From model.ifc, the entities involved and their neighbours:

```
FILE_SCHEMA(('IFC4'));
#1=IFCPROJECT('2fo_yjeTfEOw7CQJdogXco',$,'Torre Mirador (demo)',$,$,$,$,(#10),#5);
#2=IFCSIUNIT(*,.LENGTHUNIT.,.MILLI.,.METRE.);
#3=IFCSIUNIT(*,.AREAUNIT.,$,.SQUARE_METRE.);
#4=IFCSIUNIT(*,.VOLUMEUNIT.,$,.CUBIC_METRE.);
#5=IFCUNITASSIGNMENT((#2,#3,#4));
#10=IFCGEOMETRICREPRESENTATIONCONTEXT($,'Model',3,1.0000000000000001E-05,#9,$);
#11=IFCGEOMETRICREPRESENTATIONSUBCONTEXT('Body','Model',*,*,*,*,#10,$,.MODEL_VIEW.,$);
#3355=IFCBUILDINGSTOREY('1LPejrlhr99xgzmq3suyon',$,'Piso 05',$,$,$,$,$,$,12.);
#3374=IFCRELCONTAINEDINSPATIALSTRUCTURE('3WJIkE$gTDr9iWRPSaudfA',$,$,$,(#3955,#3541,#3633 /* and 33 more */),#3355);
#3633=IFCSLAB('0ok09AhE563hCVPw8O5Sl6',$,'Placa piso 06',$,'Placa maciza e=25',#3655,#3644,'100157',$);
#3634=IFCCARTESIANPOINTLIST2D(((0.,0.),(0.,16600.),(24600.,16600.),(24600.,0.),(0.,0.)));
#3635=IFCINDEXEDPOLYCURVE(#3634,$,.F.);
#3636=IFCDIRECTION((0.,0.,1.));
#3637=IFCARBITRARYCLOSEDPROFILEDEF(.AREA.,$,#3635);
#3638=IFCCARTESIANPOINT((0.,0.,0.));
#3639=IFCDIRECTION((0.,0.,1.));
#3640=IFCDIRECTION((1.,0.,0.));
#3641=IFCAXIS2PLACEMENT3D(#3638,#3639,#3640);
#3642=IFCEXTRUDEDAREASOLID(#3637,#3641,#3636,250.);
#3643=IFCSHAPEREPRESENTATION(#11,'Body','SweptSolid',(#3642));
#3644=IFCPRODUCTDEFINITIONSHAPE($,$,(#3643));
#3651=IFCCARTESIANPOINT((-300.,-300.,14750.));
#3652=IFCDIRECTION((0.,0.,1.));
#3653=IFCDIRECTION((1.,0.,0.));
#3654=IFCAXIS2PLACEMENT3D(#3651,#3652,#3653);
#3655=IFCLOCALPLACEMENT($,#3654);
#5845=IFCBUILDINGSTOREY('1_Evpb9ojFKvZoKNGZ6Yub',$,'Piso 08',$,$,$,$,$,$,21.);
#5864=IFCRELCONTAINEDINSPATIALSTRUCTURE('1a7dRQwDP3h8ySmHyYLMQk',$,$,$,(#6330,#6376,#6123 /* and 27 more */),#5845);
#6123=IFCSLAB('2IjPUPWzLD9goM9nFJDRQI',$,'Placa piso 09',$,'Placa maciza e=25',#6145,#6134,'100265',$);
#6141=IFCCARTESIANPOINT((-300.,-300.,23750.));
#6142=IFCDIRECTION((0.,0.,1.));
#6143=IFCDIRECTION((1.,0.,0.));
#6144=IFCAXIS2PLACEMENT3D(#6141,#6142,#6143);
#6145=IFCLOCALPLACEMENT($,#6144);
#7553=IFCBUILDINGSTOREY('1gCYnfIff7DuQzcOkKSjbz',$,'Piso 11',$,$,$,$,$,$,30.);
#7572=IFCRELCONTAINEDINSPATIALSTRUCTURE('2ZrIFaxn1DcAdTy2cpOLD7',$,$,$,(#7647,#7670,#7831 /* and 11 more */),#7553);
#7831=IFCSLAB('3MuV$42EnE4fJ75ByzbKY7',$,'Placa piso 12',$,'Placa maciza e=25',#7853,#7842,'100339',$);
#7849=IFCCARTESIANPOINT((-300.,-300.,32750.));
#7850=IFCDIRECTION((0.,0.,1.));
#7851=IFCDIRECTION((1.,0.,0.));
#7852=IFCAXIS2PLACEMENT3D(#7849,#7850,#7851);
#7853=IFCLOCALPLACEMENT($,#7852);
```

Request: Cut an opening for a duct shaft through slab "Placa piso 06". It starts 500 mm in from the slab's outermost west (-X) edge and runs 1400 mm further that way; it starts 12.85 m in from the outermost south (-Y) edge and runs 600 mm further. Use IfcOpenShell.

```python
import numpy as np
import ifcopenshell
import ifcopenshell.api.feature
import ifcopenshell.api.geometry
import ifcopenshell.api.root
import ifcopenshell.geom
import ifcopenshell.util.placement
import ifcopenshell.util.representation
import ifcopenshell.util.shape
import ifcopenshell.util.unit

model = ifcopenshell.open("model.ifc")
unit_scale = ifcopenshell.util.unit.calculate_unit_scale(model)
settings = ifcopenshell.geom.settings()


def volume(element):
    """Net volume in cubic metres, openings subtracted."""
    shape = ifcopenshell.geom.create_shape(settings, element)
    return ifcopenshell.util.shape.get_volume(shape.geometry)


slab = model.by_guid("0ok09AhE563hCVPw8O5Sl6")
before = volume(slab)

# Extent in the slab's own axes, in metres. The edges named are its -X and -Y sides.
slab_shape = ifcopenshell.geom.create_shape(settings, slab)
vertices = ifcopenshell.util.shape.get_vertices(slab_shape.geometry)
x_min, y_min, bottom = vertices.min(axis=0)
top = vertices[:, 2].max()

opening = ifcopenshell.api.root.create_entity(model, ifc_class="IfcOpeningElement", name="Duct shaft opening", predefined_type="OPENING")
context = ifcopenshell.util.representation.get_context(model, "Model", "Body", "MODEL_VIEW")
width, depth = 1.4, 0.6
outline = [(0.0, 0.0), (width, 0.0), (width, depth), (0.0, depth), (0.0, 0.0)]
# Overshoot both faces by 50 mm so the cut is clean.
shape = ifcopenshell.api.geometry.add_slab_representation(
    model, context=context, depth=top - bottom + 0.1, polyline=outline
)
ifcopenshell.api.geometry.assign_representation(model, product=opening, representation=shape)

matrix = ifcopenshell.util.placement.get_local_placement(slab.ObjectPlacement)
matrix[:, 3] = matrix @ np.append(np.array([x_min + 0.5, y_min + 12.85, bottom - 0.05]) / unit_scale, 1.0)
ifcopenshell.api.geometry.edit_object_placement(model, product=opening, matrix=matrix, is_si=False)
ifcopenshell.api.feature.add_feature(model, feature=opening, element=slab)

after = volume(slab)

print(f"slab volume {before:.3f} -> {after:.3f} m3")

model.write("model-out.ifc")
```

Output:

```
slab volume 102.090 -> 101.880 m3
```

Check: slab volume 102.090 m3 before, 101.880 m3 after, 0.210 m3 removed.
